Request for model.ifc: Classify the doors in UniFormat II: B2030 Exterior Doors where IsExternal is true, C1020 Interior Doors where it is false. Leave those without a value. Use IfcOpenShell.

First a look at what the model holds.

```python
import ifcopenshell
import ifcopenshell.util.element

model = ifcopenshell.open("model.ifc")
print(model.schema)
print("classifications:", [c.Name for c in model.by_type("IfcClassification")])
values = [ifcopenshell.util.element.get_pset(e, "Pset_DoorCommon", "IsExternal") for e in model.by_type("IfcDoor")]
for value in (True, False, None):
    print("IsExternal", value, values.count(value))
```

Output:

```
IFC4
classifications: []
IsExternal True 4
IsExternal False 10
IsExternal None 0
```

```python
import ifcopenshell
import ifcopenshell.api.classification
import ifcopenshell.util.element

model = ifcopenshell.open("model.ifc")

system = ifcopenshell.api.classification.add_classification(model, classification="UniFormat II")

doors = model.by_type("IfcDoor")
external = {e: ifcopenshell.util.element.get_pset(e, "Pset_DoorCommon", "IsExternal") for e in doors}
for flag, code, name in ((True, "B2030", "Exterior Doors"), (False, "C1020", "Interior Doors")):
    products = [e for e in doors if external[e] is flag]
    ifcopenshell.api.classification.add_reference(
        model, products=products, classification=system, identification=code, name=name
    )
    print(code, len(products))

model.write("model_rev.ifc")
```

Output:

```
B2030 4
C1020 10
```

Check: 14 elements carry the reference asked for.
